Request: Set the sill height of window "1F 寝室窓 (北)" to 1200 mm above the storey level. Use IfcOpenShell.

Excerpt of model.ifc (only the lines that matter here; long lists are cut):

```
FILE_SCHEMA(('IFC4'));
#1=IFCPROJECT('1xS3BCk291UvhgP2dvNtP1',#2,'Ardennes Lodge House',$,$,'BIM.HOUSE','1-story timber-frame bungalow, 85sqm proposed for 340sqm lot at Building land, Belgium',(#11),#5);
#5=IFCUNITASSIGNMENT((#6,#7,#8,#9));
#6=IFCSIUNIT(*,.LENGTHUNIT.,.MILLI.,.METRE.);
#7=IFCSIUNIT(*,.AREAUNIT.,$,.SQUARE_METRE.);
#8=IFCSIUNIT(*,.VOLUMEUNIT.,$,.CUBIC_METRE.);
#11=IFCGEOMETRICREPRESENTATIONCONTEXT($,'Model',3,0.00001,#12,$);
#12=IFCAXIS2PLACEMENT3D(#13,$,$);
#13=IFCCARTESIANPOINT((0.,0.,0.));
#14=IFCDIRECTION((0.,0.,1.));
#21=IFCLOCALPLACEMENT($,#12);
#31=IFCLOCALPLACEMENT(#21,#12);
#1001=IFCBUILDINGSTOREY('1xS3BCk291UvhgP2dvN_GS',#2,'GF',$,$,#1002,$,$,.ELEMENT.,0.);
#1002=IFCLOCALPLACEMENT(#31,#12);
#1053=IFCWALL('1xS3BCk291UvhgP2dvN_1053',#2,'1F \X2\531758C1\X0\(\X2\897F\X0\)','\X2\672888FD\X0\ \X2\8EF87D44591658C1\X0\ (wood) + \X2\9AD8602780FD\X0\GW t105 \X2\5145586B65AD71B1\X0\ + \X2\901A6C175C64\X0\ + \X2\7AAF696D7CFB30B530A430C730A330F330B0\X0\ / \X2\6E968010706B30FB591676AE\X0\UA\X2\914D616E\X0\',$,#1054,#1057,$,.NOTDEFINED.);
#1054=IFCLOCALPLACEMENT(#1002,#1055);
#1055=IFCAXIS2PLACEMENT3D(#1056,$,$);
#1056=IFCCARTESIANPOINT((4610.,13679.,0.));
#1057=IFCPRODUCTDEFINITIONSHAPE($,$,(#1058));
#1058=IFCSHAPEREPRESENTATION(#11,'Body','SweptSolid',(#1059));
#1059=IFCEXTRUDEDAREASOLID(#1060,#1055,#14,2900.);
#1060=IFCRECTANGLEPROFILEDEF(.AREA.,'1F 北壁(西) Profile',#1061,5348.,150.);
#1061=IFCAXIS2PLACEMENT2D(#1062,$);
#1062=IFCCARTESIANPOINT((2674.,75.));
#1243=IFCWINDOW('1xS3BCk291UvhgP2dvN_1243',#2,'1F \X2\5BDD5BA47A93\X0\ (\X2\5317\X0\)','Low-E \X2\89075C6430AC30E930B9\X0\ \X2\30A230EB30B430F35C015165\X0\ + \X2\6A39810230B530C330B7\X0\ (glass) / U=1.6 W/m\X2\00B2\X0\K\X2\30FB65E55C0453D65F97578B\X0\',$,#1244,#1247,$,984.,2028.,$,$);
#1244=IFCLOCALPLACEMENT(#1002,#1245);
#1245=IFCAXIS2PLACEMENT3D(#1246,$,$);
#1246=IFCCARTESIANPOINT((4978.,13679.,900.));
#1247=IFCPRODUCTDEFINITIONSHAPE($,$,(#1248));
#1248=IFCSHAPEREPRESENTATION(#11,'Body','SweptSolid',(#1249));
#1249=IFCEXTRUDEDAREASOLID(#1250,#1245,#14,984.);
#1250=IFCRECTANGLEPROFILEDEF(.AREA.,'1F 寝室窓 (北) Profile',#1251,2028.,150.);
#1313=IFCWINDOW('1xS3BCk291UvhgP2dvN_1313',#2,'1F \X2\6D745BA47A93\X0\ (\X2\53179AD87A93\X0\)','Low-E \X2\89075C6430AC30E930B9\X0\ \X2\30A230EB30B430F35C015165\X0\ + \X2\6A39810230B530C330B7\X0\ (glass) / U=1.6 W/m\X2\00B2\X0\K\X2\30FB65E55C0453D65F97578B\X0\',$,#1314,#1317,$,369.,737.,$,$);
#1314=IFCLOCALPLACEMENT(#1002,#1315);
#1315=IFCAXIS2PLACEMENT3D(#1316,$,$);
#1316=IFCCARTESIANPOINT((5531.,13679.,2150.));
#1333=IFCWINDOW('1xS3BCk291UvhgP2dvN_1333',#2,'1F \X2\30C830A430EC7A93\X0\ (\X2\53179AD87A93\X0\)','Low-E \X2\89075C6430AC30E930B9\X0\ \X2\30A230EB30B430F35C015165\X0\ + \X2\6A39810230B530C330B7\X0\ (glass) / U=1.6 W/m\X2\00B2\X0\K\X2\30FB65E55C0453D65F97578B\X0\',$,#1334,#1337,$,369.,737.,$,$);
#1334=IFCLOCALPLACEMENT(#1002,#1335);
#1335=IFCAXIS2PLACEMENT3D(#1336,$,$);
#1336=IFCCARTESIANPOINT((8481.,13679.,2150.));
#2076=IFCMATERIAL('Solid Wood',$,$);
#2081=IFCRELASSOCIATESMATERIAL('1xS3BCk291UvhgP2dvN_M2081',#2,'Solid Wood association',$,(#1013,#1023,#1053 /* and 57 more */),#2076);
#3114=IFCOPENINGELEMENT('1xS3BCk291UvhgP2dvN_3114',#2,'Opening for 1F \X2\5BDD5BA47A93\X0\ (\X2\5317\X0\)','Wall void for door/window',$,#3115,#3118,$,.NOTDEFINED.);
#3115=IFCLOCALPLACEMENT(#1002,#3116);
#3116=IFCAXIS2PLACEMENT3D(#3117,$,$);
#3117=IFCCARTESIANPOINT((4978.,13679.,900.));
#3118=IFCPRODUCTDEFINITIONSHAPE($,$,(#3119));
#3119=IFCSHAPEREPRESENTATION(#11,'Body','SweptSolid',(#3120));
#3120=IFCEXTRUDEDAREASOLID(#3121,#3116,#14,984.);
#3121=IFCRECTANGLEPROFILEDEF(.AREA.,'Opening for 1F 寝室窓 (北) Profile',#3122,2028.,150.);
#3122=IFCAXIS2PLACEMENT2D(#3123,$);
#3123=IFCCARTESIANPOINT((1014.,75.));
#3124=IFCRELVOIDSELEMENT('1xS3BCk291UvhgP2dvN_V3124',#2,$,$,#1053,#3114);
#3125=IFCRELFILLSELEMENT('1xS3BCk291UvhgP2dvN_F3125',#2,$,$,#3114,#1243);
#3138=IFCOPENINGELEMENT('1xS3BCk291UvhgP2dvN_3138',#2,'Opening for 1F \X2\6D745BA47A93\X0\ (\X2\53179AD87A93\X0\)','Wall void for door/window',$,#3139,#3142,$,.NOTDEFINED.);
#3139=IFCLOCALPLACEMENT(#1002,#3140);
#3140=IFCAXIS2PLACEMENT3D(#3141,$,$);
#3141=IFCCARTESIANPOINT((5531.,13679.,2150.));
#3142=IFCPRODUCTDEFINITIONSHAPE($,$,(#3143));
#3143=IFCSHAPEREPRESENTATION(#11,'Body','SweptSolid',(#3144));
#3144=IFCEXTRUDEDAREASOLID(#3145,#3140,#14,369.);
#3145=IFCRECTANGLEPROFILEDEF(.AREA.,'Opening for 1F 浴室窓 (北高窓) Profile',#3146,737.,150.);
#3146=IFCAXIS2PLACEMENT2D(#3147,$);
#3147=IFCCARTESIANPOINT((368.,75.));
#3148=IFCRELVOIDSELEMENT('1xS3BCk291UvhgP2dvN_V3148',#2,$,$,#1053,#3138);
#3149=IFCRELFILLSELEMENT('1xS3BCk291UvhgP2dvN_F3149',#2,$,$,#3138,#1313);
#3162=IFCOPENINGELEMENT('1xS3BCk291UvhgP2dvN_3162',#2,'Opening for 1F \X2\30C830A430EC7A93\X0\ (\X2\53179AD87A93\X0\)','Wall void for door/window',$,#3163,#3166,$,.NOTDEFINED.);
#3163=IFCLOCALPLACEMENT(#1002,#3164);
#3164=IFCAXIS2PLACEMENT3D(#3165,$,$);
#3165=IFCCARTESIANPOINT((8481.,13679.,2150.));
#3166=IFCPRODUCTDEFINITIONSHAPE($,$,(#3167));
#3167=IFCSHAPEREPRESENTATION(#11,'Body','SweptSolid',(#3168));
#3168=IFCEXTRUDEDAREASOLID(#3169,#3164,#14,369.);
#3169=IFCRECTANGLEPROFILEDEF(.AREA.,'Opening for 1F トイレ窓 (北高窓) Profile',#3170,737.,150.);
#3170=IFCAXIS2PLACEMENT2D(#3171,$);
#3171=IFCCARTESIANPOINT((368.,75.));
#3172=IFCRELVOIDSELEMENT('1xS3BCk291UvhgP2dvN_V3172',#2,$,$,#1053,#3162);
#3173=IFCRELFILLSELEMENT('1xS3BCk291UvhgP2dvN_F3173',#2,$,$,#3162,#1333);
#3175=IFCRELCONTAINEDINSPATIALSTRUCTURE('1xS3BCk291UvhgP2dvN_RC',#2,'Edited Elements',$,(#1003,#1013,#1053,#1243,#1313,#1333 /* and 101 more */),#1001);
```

```python
import numpy as np
import ifcopenshell
import ifcopenshell.api.geometry
import ifcopenshell.geom
import ifcopenshell.util.element
import ifcopenshell.util.placement
import ifcopenshell.util.shape
import ifcopenshell.util.unit

model = ifcopenshell.open("model.ifc")
unit_scale = ifcopenshell.util.unit.calculate_unit_scale(model)

window = model.by_id(1243)
opening = window.FillsVoids[0].RelatingOpeningElement
storey = ifcopenshell.util.element.get_container(window, ifc_class="IfcBuildingStorey")
level = ifcopenshell.util.placement.get_local_placement(storey.ObjectPlacement)[2, 3]

# The opening's origin need not be at the sill, so measure its lowest point.
shape = ifcopenshell.geom.create_shape(ifcopenshell.geom.settings(), opening)
bottom = ifcopenshell.util.shape.get_shape_bottom_elevation(shape, shape.geometry) / unit_scale
dz = level + 1.2 / unit_scale - bottom

shift = np.array([0.0, 0.0, dz])
# The window is not placed relative to its opening, so move both.
for product in (opening, window):
    matrix = ifcopenshell.util.placement.get_local_placement(product.ObjectPlacement)
    matrix[:3, 3] += shift
    ifcopenshell.api.geometry.edit_object_placement(model, product=product, matrix=matrix, is_si=False)

print(f"moved by {dz * unit_scale:+.3f} m")

model.write("model_v2.ifc")
```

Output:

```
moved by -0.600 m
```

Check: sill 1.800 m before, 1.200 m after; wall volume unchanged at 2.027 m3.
